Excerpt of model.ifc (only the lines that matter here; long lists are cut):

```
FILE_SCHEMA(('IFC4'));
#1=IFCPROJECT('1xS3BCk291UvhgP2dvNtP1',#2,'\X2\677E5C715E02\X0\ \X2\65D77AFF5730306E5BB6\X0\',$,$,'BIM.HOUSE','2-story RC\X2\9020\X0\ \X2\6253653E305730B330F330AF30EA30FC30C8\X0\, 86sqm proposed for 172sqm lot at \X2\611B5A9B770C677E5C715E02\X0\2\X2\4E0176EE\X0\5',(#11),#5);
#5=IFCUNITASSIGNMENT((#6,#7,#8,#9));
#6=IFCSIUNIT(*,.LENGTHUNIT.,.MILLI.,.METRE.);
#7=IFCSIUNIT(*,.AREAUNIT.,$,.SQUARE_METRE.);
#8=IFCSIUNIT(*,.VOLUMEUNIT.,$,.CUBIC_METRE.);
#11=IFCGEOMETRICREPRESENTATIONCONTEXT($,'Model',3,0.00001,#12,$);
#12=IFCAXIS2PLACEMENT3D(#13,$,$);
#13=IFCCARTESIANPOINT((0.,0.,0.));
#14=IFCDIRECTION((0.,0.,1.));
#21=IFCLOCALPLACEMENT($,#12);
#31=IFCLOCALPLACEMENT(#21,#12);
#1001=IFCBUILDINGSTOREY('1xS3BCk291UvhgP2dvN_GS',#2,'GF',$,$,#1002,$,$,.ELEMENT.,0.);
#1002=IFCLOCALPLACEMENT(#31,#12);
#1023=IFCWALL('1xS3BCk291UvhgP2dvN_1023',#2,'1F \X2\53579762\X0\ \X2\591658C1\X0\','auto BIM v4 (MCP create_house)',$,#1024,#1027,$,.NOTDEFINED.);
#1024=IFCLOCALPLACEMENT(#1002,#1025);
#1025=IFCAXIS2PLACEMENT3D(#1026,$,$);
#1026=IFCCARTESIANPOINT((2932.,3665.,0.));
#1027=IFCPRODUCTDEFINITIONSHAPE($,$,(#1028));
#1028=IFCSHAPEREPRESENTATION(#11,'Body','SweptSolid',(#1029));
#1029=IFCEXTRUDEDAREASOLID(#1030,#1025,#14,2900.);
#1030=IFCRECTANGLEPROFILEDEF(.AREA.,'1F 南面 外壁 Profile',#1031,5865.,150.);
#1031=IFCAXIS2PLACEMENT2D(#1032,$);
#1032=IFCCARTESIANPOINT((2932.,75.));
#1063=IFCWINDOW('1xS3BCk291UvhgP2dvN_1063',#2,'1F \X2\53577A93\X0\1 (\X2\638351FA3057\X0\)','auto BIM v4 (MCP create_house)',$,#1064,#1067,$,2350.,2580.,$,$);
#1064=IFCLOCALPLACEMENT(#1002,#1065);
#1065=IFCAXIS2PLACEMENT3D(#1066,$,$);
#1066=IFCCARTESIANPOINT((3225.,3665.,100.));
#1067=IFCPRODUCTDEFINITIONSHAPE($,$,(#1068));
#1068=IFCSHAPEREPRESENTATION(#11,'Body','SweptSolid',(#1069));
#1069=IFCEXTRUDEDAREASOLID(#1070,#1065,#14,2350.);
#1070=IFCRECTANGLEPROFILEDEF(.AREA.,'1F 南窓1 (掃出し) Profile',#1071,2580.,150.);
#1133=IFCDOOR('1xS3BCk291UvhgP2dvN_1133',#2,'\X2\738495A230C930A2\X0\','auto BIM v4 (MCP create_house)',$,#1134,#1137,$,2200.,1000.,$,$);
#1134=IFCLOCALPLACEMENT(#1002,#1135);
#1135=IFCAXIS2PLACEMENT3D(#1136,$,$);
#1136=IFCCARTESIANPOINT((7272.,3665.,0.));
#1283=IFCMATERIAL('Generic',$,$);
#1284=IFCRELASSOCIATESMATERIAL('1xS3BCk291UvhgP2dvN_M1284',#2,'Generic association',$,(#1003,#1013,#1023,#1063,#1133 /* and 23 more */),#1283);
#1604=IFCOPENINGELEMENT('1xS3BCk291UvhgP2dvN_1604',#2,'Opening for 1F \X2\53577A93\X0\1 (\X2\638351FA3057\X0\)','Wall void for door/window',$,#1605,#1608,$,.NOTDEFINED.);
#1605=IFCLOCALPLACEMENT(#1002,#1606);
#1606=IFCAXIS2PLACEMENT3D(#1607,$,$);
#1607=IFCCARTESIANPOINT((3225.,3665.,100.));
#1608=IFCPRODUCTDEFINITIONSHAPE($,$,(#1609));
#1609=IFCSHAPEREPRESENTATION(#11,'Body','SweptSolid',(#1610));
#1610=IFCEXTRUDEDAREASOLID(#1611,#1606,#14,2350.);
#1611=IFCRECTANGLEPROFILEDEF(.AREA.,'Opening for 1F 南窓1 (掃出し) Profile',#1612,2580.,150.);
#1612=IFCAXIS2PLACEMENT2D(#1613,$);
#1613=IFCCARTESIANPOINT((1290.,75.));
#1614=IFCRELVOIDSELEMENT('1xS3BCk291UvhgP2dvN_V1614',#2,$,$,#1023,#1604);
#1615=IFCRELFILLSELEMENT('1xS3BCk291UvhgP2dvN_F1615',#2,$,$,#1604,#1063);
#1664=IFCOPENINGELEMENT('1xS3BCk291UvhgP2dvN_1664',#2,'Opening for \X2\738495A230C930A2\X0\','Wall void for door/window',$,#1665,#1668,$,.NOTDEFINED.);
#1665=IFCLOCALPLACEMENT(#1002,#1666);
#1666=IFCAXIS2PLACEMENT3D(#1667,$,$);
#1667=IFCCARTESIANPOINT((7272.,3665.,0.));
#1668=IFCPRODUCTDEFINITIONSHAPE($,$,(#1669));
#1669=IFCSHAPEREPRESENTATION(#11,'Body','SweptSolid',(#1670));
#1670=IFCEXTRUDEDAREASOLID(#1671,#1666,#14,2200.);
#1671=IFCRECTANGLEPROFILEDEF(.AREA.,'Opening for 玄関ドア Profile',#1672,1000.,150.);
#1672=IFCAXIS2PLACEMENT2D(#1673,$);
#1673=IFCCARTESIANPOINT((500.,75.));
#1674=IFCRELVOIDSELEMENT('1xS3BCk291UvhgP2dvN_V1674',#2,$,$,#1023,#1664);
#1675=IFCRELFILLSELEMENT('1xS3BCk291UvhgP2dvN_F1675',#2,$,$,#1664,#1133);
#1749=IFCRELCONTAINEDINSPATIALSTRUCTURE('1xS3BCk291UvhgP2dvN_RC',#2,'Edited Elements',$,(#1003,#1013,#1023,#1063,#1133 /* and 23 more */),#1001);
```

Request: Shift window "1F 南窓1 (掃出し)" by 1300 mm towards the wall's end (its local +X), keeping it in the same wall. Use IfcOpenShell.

```python
import ifcopenshell
import ifcopenshell.api.geometry
import ifcopenshell.util.placement
import ifcopenshell.util.unit

model = ifcopenshell.open("model.ifc")
unit_scale = ifcopenshell.util.unit.calculate_unit_scale(model)

window = model.by_id(1063)
opening = window.FillsVoids[0].RelatingOpeningElement
wall = opening.VoidsElements[0].RelatingBuildingElement

wall_matrix = ifcopenshell.util.placement.get_local_placement(wall.ObjectPlacement)
shift = wall_matrix[:3, 0] * 1.3 / unit_scale
before = ifcopenshell.util.placement.get_local_placement(window.ObjectPlacement)[:3, 3].copy()

# The window is not placed relative to its opening, so move both.
for product in (opening, window):
    matrix = ifcopenshell.util.placement.get_local_placement(product.ObjectPlacement)
    matrix[:3, 3] += shift
    ifcopenshell.api.geometry.edit_object_placement(model, product=product, matrix=matrix, is_si=False)

after = ifcopenshell.util.placement.get_local_placement(window.ObjectPlacement)[:3, 3]
print("window moved by", (after - before).round(3) + 0.0)

model.write("model_edited.ifc")
```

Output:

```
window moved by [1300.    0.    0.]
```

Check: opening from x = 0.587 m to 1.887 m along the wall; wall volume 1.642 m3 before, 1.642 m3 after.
